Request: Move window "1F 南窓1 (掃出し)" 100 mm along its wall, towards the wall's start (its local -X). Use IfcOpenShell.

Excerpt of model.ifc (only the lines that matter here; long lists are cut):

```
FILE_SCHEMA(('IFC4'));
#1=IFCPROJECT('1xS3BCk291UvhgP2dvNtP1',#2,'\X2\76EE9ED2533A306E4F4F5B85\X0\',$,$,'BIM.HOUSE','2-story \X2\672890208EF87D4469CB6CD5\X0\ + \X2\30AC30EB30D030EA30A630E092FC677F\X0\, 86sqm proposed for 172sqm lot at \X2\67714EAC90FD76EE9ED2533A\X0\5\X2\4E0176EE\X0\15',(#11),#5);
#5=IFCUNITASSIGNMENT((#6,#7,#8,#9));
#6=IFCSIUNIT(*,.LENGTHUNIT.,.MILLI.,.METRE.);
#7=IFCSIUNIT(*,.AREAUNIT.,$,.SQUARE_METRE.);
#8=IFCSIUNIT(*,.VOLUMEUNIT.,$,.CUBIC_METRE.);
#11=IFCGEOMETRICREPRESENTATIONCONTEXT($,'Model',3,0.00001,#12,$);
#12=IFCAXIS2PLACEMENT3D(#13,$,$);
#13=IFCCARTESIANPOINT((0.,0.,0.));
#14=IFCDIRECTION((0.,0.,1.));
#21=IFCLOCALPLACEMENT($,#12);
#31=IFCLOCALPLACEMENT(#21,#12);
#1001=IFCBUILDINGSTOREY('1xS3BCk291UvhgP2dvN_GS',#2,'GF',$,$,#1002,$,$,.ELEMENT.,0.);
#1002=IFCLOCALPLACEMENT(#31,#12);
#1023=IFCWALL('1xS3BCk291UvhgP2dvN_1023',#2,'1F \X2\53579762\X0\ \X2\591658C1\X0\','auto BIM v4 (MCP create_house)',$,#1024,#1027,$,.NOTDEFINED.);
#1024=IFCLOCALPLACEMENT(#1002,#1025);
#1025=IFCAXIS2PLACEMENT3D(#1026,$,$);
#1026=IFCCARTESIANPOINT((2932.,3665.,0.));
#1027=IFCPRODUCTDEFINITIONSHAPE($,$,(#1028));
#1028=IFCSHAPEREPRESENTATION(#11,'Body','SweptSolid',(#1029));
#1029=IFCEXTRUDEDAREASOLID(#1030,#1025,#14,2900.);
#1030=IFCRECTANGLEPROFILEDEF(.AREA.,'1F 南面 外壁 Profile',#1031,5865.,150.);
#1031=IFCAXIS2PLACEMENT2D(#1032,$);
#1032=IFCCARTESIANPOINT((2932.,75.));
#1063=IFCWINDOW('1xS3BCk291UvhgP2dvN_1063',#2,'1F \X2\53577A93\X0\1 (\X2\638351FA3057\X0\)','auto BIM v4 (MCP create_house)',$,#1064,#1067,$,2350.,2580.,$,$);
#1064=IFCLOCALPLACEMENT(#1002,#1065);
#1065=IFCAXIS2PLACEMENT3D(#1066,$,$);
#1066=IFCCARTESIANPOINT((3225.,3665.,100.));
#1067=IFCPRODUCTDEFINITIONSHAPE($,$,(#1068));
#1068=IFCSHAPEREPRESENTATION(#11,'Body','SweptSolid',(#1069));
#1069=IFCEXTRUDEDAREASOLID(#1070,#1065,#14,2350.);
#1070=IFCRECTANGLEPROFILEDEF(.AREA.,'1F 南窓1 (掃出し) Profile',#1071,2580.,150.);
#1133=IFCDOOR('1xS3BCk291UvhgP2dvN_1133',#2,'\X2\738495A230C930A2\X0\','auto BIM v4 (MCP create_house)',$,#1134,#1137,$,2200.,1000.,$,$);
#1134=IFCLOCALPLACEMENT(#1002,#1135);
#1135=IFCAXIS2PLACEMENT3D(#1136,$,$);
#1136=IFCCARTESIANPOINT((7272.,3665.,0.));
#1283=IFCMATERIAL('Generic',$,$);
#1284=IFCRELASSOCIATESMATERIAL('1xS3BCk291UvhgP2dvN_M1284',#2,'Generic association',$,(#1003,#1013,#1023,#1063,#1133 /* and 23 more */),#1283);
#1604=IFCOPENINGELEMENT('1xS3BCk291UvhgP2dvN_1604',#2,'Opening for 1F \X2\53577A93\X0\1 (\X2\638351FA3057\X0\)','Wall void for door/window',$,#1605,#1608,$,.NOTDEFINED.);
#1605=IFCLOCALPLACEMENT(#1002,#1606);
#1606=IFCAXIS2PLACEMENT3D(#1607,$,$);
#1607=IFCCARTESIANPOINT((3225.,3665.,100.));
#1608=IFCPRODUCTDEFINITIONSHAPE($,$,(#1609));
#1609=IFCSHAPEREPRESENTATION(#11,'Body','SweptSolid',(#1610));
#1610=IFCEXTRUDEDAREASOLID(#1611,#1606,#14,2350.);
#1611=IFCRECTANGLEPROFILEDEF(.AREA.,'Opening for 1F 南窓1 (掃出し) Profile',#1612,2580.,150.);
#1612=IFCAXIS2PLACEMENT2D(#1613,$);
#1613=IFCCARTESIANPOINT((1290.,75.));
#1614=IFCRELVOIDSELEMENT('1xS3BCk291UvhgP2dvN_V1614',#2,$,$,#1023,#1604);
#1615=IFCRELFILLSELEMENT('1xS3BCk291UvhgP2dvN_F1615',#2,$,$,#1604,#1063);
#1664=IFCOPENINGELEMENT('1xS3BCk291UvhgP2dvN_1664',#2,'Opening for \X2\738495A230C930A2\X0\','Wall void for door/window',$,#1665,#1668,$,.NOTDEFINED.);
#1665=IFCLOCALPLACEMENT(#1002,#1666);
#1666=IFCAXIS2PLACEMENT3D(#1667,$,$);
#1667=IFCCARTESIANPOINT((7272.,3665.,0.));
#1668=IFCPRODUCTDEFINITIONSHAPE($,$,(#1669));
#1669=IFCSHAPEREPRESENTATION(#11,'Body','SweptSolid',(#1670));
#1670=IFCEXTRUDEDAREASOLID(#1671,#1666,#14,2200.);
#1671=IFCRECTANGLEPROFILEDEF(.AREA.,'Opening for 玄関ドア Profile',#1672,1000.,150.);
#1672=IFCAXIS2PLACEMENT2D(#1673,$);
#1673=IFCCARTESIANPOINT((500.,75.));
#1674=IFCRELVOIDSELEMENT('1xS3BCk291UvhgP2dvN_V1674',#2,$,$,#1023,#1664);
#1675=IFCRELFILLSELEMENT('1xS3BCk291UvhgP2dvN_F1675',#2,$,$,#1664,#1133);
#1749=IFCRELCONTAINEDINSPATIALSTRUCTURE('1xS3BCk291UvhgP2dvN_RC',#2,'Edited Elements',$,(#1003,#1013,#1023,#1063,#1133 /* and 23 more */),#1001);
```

```python
import ifcopenshell
import ifcopenshell.api.geometry
import ifcopenshell.util.placement

model = ifcopenshell.open("model.ifc")

window = model.by_id(1063)
opening = window.FillsVoids[0].RelatingOpeningElement
wall = opening.VoidsElements[0].RelatingBuildingElement

wall_matrix = ifcopenshell.util.placement.get_local_placement(wall.ObjectPlacement)
shift = wall_matrix[:3, 0] * -100.0
before = ifcopenshell.util.placement.get_local_placement(window.ObjectPlacement)[:3, 3].copy()

# The window is not placed relative to its opening, so move both.
for product in (opening, window):
    matrix = ifcopenshell.util.placement.get_local_placement(product.ObjectPlacement)
    matrix[:3, 3] += shift
    ifcopenshell.api.geometry.edit_object_placement(model, product=product, matrix=matrix, is_si=False)

after = ifcopenshell.util.placement.get_local_placement(window.ObjectPlacement)[:3, 3]
print("window moved by", (after - before).round(3) + 0.0)

model.write("model_rev.ifc")
```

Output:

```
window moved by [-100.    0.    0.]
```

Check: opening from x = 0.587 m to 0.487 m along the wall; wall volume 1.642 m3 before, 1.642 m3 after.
